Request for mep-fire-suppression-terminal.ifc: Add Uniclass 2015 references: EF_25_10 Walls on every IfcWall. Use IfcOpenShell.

First a look at what the model holds.

```python
import ifcopenshell

model = ifcopenshell.open("mep-fire-suppression-terminal.ifc")
print(model.schema)
print("classifications:", [c.Name for c in model.by_type("IfcClassification")])
for ifc_class in ("IfcDoor", "IfcRoof", "IfcStair", "IfcWall", "IfcWindow"):
    print(ifc_class, len(model.by_type(ifc_class)))
```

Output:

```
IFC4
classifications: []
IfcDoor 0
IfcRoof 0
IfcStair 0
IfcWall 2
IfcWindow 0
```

```python
import ifcopenshell
import ifcopenshell.api.classification

model = ifcopenshell.open("mep-fire-suppression-terminal.ifc")

system = ifcopenshell.api.classification.add_classification(model, classification="Uniclass 2015")

codes = {
    "IfcWall": ("EF_25_10", "Walls"),
}
for ifc_class, (code, name) in codes.items():
    products = model.by_type(ifc_class)
    ifcopenshell.api.classification.add_reference(
        model, products=products, classification=system, identification=code, name=name
    )
    print(code, len(products))

model.write("mep-fire-suppression-terminal_edited.ifc")
```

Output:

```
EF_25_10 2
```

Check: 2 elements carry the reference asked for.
